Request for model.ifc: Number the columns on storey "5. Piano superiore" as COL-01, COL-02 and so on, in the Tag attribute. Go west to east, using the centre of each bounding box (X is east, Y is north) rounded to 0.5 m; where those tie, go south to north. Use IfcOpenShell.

First a look at what the model holds.

```python
import ifcopenshell
import ifcopenshell.util.element
import ifcopenshell.util.placement

model = ifcopenshell.open("model.ifc")
print(model.schema)
storey = next(s for s in model.by_type("IfcBuildingStorey") if s.Name == "5. Piano superiore")
columns = [e for e in ifcopenshell.util.element.get_decomposition(storey) if e.is_a("IfcColumn")]
for e in sorted(columns, key=lambda e: e.id()):
    origin = ifcopenshell.util.placement.get_local_placement(e.ObjectPlacement)[:3, 3]
    print(e.id(), e.Tag, e.Name, origin.round(2) + 0.0, sep=" | ")
```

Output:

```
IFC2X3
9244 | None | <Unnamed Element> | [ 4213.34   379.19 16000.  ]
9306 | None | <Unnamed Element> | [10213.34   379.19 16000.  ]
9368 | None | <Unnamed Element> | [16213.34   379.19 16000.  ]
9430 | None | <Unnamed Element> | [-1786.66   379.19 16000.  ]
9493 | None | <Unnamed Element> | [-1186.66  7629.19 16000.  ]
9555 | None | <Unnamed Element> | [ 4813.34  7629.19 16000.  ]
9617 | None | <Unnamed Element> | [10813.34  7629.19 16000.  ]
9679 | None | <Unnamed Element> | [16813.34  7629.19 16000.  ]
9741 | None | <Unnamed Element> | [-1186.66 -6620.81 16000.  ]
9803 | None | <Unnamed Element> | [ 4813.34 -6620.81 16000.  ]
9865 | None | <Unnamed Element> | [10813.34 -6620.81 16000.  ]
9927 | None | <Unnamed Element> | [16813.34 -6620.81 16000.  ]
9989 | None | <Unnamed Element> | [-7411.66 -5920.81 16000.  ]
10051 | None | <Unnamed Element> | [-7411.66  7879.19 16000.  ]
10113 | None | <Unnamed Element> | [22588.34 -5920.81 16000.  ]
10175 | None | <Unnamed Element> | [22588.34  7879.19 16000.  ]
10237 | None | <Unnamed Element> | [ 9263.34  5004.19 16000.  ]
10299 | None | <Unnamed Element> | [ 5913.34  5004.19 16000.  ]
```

```python
import ifcopenshell
import ifcopenshell.geom
import ifcopenshell.util.element
import ifcopenshell.util.shape

model = ifcopenshell.open("model.ifc")
settings = ifcopenshell.geom.settings()
settings.set("use-world-coords", True)


def centre(element):
    shape = ifcopenshell.geom.create_shape(settings, element)
    return ifcopenshell.util.shape.get_bbox_centroid(shape.geometry)


storey = next(s for s in model.by_type("IfcBuildingStorey") if s.Name == "5. Piano superiore")
columns = [e for e in ifcopenshell.util.element.get_decomposition(storey) if e.is_a("IfcColumn")]

# Insertion points can sit at a corner or the storey origin, so sort by the geometry (in metres).
centres = {e: centre(e) for e in columns}
columns.sort(key=lambda e: (round(centres[e][0] / 0.5), centres[e][1]))

for i, e in enumerate(columns, start=1):
    number = f"COL-{i:02d}"
    e.Tag = number
    print(e.id(), number)

model.write("model_v2.ifc")
```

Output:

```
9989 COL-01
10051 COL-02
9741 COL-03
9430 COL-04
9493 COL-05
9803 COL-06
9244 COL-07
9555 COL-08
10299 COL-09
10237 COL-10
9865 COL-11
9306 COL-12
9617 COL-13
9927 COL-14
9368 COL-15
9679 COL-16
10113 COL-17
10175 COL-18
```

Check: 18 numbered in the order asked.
